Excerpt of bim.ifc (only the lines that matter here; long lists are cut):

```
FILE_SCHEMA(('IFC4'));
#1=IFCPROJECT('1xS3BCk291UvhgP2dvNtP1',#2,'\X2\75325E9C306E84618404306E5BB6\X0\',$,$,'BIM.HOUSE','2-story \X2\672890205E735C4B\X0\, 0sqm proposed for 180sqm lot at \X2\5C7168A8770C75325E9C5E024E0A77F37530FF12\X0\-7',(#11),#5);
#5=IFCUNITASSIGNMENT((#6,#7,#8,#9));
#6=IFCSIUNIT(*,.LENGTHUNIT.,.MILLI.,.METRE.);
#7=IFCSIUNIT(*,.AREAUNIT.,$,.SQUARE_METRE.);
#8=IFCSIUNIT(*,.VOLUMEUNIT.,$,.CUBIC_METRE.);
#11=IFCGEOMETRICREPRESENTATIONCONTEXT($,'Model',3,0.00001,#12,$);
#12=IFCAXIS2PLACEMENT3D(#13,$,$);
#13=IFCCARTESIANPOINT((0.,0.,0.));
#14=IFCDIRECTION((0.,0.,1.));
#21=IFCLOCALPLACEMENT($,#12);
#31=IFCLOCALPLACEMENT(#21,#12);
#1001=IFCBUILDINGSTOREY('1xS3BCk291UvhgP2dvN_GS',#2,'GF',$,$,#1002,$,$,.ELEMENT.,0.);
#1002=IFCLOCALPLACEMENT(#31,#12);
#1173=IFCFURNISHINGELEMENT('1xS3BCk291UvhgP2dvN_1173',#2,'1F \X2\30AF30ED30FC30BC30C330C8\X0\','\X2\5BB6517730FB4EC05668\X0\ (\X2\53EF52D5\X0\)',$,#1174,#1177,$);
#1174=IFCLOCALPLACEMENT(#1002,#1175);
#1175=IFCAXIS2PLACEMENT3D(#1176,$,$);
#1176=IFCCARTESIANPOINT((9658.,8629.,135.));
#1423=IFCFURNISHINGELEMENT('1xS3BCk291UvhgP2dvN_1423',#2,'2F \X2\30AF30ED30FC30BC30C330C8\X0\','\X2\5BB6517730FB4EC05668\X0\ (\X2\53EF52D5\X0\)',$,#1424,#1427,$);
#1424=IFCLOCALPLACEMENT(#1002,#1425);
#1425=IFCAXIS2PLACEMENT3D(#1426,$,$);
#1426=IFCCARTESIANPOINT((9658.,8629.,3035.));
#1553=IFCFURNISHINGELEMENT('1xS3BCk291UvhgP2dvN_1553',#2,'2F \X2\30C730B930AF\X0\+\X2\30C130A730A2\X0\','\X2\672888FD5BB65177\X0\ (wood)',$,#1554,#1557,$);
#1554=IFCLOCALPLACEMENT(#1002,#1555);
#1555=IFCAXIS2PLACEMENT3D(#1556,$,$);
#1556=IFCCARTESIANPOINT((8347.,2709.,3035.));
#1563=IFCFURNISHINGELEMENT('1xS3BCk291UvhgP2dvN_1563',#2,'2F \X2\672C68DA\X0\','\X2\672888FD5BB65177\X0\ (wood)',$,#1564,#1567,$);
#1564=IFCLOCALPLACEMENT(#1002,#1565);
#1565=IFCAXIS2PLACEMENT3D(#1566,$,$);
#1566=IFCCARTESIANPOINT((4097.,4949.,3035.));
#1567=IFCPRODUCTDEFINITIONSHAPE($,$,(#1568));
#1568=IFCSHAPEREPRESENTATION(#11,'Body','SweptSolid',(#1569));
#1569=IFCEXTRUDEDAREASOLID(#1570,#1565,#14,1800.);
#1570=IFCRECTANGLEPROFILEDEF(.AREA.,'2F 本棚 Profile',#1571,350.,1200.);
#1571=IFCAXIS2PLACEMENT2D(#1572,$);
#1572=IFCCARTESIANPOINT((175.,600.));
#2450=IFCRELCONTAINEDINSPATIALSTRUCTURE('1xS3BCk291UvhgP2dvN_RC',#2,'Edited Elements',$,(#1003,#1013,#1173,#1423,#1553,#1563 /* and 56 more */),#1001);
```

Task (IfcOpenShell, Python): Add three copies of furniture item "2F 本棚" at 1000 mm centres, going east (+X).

```python
import numpy as np
import ifcopenshell
import ifcopenshell.api.geometry
import ifcopenshell.api.root
import ifcopenshell.util.element
import ifcopenshell.util.placement

model = ifcopenshell.open("bim.ifc")


def reuse_history(source, copy):
    """copy_class also copies each property set's owner history, people and application; keep the originals."""
    for rel in copy.IsDefinedBy:
        if rel.is_a("IfcRelDefinesByProperties") and (history := rel.RelatingPropertyDefinition.OwnerHistory):
            rel.RelatingPropertyDefinition.OwnerHistory = source.OwnerHistory
            ifcopenshell.util.element.remove_deep2(model, history)


source = model.by_id(1563)
base = ifcopenshell.util.placement.get_local_placement(source.ObjectPlacement)
step = np.array([1.0, 0.0, 0.0]) * 1000.0

for i in range(1, 4):
    copy = ifcopenshell.api.root.copy_class(model, product=source)
    copy.Representation = ifcopenshell.util.element.copy_deep(
        model, source.Representation, exclude=["IfcGeometricRepresentationContext", "IfcRepresentationMap"]
    )
    reuse_history(source, copy)
    matrix = base.copy()
    matrix[:3, 3] += i * step
    print("added at", matrix[:3, 3].round(3) + 0.0)
    ifcopenshell.api.geometry.edit_object_placement(model, product=copy, matrix=matrix, is_si=False)

model.write("bim-out.ifc")
```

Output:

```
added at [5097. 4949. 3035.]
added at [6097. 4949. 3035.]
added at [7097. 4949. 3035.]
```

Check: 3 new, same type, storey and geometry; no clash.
